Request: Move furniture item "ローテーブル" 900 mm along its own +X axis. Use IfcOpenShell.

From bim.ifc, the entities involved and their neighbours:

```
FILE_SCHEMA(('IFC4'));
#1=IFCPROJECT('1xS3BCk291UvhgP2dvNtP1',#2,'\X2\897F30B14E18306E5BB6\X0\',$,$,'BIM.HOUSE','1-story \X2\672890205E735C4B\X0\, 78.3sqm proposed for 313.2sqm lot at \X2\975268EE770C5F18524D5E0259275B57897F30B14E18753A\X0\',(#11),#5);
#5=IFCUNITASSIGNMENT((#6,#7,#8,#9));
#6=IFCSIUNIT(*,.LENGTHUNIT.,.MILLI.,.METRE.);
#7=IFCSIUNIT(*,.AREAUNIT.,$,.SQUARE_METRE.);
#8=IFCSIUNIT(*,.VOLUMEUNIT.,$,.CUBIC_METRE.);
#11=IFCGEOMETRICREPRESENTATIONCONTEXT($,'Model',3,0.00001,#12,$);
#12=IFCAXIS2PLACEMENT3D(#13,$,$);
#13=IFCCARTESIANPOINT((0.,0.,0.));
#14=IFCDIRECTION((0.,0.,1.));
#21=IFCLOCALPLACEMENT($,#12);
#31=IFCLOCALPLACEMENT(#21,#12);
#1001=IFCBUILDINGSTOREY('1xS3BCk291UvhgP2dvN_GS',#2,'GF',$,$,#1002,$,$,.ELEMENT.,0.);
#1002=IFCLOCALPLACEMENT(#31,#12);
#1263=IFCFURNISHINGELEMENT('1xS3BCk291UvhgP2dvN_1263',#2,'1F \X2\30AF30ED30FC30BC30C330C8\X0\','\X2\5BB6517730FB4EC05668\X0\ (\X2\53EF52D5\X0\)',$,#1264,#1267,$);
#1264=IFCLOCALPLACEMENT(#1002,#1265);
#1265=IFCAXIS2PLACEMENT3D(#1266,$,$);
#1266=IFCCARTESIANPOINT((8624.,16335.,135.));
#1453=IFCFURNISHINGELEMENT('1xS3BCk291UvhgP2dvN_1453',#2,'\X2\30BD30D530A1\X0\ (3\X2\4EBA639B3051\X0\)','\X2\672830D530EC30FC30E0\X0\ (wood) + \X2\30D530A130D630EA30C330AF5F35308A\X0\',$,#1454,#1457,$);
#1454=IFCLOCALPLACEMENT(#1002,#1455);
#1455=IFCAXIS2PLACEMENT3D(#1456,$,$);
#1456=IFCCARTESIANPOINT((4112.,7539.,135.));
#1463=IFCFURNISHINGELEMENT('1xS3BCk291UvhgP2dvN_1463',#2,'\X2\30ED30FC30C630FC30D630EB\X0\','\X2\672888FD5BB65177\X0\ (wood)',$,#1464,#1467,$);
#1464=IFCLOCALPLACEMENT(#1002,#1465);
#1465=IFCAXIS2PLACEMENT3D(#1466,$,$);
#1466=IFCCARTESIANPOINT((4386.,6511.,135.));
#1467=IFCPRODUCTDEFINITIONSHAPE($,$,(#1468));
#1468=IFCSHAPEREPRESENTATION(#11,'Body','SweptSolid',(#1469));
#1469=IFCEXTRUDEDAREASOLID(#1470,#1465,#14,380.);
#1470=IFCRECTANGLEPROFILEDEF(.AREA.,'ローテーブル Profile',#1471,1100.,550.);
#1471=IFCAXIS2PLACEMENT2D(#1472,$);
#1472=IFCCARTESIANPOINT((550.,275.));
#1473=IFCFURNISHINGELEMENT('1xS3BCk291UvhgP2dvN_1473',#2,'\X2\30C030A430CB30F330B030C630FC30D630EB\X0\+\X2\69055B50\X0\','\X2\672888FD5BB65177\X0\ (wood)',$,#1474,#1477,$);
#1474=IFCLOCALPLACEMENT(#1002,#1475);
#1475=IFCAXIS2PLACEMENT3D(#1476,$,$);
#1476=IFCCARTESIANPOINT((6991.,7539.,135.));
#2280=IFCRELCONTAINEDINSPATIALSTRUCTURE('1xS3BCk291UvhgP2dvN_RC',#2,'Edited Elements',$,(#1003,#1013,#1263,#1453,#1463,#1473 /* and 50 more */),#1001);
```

```python
import ifcopenshell
import ifcopenshell.api.geometry
import ifcopenshell.util.placement

model = ifcopenshell.open("bim.ifc")

item = model.by_guid("1xS3BCk291UvhgP2dvN_1463")
matrix = ifcopenshell.util.placement.get_local_placement(item.ObjectPlacement)
matrix[:3, 3] += matrix[:3, 0] * 900.0
ifcopenshell.api.geometry.edit_object_placement(model, product=item, matrix=matrix, is_si=False)

print(ifcopenshell.util.placement.get_local_placement(item.ObjectPlacement).round(3) + 0.0)

model.write("bim_rev.ifc")
```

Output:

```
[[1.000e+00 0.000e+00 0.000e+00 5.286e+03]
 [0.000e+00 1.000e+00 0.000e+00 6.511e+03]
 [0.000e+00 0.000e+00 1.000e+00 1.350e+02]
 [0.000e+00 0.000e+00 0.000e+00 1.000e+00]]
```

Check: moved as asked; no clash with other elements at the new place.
